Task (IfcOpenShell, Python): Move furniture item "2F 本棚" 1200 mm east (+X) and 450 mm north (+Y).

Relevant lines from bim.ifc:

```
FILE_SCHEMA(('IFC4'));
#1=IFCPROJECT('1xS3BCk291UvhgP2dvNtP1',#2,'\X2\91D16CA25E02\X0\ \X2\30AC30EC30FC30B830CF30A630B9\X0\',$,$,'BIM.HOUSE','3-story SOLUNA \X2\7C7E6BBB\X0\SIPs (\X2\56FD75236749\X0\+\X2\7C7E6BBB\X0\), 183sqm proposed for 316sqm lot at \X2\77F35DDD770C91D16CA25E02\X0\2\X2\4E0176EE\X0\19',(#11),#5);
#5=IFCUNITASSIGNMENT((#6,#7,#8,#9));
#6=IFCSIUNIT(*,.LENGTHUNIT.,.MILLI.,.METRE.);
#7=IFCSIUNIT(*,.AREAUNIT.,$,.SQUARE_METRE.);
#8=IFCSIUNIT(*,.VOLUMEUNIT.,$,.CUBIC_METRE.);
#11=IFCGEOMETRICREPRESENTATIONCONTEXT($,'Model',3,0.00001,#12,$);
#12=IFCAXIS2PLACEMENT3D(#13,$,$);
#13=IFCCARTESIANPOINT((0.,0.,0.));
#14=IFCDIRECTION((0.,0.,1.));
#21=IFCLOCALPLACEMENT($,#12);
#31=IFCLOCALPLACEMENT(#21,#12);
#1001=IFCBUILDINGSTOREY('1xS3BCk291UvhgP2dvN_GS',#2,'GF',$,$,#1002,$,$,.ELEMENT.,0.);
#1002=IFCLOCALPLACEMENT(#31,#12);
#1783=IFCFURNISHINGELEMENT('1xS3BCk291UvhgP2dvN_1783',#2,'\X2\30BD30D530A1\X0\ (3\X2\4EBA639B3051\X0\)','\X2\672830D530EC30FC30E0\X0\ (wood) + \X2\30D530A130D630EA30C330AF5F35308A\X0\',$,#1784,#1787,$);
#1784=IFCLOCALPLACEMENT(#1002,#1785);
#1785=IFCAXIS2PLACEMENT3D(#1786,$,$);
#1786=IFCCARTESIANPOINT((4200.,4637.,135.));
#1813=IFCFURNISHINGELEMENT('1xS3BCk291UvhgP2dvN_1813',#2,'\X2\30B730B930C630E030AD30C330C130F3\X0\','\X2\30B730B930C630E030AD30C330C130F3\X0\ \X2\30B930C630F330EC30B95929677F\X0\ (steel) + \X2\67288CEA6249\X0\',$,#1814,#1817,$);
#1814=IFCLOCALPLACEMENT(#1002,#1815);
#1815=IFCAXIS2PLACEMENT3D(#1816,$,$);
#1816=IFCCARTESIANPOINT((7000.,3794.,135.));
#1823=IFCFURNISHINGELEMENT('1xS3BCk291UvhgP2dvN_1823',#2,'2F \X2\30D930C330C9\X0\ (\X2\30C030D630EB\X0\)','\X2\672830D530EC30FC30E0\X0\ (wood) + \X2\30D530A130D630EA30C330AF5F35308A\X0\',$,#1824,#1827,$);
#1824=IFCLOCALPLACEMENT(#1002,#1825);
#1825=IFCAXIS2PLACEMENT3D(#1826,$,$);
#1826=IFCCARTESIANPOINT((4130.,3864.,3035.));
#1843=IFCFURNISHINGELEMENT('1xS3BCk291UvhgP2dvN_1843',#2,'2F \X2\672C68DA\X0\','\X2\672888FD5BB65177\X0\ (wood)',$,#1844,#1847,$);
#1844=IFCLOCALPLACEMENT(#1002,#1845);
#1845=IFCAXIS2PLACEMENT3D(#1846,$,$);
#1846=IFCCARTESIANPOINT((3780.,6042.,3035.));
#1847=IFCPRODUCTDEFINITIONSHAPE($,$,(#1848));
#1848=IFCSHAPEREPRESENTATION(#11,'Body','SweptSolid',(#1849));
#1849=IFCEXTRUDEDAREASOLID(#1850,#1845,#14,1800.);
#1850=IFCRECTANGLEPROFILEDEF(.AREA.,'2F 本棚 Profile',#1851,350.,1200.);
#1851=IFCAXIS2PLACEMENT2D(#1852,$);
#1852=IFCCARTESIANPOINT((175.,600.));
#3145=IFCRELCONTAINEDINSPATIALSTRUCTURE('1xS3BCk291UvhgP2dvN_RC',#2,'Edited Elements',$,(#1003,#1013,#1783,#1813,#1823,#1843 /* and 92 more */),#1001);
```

```python
import ifcopenshell
import ifcopenshell.api.geometry
import ifcopenshell.util.placement

model = ifcopenshell.open("bim.ifc")

item = model.by_guid("1xS3BCk291UvhgP2dvN_1843")
matrix = ifcopenshell.util.placement.get_local_placement(item.ObjectPlacement)
matrix[0, 3] += 1200.0
matrix[1, 3] += 450.0
ifcopenshell.api.geometry.edit_object_placement(model, product=item, matrix=matrix, is_si=False)

print(ifcopenshell.util.placement.get_local_placement(item.ObjectPlacement).round(3) + 0.0)

model.write("bim-out.ifc")
```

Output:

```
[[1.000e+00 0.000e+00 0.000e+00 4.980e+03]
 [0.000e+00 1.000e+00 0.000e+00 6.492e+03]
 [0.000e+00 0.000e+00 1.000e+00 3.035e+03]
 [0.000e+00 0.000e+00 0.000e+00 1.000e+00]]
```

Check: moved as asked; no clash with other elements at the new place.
